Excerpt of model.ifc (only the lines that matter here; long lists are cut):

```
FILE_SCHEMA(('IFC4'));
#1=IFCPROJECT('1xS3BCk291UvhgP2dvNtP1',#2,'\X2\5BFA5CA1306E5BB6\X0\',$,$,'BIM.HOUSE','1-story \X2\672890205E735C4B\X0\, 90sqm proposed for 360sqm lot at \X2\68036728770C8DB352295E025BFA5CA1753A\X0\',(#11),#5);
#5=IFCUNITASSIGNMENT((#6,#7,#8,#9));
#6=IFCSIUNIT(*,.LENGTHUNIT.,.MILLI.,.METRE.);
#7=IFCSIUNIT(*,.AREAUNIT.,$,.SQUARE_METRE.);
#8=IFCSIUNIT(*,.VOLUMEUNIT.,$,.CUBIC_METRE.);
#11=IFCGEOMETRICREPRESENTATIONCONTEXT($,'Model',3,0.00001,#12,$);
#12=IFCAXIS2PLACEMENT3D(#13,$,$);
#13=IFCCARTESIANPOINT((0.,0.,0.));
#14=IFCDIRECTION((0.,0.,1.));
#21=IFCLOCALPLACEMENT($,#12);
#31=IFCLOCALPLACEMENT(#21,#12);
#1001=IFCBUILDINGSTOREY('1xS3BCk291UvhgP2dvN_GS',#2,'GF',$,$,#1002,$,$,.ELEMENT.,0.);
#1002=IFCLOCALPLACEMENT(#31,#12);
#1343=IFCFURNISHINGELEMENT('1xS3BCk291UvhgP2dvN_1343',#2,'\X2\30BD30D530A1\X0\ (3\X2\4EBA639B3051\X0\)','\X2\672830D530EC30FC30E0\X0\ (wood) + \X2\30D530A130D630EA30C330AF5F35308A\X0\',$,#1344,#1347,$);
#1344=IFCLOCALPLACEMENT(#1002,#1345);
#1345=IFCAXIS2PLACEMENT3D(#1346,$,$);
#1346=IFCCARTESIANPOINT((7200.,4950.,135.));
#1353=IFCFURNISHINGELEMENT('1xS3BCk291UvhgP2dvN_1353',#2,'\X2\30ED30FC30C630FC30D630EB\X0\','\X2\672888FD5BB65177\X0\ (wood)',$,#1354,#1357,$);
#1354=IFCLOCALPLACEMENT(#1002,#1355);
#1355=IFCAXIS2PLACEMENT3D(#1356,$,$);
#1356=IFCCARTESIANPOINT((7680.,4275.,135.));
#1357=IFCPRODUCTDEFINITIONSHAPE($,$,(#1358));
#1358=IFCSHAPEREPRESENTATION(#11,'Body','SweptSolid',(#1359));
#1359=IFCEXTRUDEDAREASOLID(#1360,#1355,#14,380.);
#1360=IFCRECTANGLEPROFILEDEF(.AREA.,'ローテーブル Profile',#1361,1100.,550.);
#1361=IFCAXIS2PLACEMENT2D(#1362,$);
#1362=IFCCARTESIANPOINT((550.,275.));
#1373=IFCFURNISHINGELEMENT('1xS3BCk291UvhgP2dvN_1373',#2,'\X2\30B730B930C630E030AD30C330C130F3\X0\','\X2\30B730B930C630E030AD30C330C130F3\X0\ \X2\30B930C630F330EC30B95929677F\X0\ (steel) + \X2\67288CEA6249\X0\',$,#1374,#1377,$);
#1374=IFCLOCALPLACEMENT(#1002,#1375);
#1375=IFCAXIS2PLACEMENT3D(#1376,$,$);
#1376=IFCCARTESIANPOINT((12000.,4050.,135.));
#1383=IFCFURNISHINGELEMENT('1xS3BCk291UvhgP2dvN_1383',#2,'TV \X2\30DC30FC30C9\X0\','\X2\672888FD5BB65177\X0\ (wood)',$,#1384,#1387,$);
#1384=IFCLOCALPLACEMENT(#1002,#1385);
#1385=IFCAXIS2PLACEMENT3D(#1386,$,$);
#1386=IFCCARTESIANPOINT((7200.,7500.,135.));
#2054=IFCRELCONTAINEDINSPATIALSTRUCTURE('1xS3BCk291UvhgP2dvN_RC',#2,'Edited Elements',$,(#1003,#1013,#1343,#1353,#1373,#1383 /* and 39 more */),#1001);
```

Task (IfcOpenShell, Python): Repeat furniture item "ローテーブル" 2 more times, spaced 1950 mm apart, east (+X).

```python
import numpy as np
import ifcopenshell
import ifcopenshell.api.geometry
import ifcopenshell.api.root
import ifcopenshell.util.element
import ifcopenshell.util.placement

model = ifcopenshell.open("model.ifc")


def reuse_history(source, copy):
    """copy_class also copies each property set's owner history, people and application; keep the originals."""
    for rel in copy.IsDefinedBy:
        if rel.is_a("IfcRelDefinesByProperties") and (history := rel.RelatingPropertyDefinition.OwnerHistory):
            rel.RelatingPropertyDefinition.OwnerHistory = source.OwnerHistory
            ifcopenshell.util.element.remove_deep2(model, history)


source = model.by_guid("1xS3BCk291UvhgP2dvN_1353")
base = ifcopenshell.util.placement.get_local_placement(source.ObjectPlacement)
step = np.array([1.0, 0.0, 0.0]) * 1950.0

for i in range(1, 3):
    copy = ifcopenshell.api.root.copy_class(model, product=source)
    copy.Representation = ifcopenshell.util.element.copy_deep(
        model, source.Representation, exclude=["IfcGeometricRepresentationContext", "IfcRepresentationMap"]
    )
    reuse_history(source, copy)
    matrix = base.copy()
    matrix[:3, 3] += i * step
    print("added at", matrix[:3, 3].round(3) + 0.0)
    ifcopenshell.api.geometry.edit_object_placement(model, product=copy, matrix=matrix, is_si=False)

model.write("model_updated.ifc")
```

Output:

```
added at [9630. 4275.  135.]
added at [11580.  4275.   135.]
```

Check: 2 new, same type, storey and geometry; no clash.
